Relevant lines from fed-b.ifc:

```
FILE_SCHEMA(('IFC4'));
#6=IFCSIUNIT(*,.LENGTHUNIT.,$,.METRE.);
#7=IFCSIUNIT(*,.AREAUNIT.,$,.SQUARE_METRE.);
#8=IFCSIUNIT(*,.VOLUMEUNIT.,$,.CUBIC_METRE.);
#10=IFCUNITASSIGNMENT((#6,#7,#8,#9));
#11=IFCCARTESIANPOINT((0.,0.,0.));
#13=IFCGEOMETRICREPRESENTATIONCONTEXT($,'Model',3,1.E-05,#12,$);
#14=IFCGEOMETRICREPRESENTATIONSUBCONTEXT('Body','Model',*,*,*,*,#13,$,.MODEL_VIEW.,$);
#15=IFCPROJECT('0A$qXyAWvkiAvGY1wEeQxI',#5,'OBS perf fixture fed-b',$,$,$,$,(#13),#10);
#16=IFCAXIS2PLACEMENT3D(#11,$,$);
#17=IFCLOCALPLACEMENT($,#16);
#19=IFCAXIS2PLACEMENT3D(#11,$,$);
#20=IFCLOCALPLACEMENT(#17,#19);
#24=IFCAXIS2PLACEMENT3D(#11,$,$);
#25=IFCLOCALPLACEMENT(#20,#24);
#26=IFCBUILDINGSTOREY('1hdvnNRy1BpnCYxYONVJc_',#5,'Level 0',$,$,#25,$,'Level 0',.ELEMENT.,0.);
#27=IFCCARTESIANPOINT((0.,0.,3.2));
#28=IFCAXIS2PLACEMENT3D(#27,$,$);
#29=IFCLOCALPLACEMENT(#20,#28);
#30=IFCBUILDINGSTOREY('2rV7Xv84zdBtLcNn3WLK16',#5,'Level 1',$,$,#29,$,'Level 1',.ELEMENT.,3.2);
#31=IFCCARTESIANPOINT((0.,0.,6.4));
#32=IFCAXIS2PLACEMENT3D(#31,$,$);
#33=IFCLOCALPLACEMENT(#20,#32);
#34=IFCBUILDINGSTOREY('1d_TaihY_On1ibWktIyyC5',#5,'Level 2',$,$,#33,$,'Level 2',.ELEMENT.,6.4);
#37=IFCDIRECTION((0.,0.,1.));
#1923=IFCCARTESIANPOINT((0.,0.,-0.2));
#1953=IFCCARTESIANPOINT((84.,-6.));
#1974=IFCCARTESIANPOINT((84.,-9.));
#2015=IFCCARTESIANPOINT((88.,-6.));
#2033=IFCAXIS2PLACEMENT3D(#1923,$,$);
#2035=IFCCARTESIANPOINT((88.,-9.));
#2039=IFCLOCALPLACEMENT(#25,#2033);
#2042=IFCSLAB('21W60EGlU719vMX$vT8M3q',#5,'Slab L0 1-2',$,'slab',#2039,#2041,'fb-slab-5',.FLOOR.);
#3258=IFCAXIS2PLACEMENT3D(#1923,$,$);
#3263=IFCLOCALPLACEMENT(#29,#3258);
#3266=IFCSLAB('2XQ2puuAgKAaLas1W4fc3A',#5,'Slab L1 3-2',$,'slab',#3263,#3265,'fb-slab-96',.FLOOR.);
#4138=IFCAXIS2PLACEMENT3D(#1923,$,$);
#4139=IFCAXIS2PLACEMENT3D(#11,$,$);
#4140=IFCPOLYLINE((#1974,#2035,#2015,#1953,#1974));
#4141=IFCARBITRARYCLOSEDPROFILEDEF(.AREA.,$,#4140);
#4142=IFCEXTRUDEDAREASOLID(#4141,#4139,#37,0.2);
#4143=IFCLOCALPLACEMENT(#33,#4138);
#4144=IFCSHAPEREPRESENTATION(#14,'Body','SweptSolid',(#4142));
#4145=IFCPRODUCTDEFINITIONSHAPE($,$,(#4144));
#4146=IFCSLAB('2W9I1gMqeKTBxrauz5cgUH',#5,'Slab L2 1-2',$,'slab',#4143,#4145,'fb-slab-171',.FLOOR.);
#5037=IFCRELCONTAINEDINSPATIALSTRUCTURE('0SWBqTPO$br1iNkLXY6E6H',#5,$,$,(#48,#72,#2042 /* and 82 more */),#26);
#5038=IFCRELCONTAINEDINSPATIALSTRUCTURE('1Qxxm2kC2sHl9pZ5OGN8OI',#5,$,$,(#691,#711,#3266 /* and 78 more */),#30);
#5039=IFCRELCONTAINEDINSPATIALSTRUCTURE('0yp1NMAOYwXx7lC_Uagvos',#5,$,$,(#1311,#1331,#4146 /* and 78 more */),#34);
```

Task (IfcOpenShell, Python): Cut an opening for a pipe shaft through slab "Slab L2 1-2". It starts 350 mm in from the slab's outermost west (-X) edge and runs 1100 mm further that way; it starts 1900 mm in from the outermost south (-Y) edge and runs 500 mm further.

```python
import numpy as np
import ifcopenshell
import ifcopenshell.api.feature
import ifcopenshell.api.geometry
import ifcopenshell.api.root
import ifcopenshell.geom
import ifcopenshell.util.placement
import ifcopenshell.util.representation
import ifcopenshell.util.shape
import ifcopenshell.util.unit

model = ifcopenshell.open("fed-b.ifc")
unit_scale = ifcopenshell.util.unit.calculate_unit_scale(model)
settings = ifcopenshell.geom.settings()


def volume(element):
    """Net volume in cubic metres, openings subtracted."""
    shape = ifcopenshell.geom.create_shape(settings, element)
    return ifcopenshell.util.shape.get_volume(shape.geometry)


slab = model.by_guid("2W9I1gMqeKTBxrauz5cgUH")
before = volume(slab)

# Extent in the slab's own axes, in metres. The edges named are its -X and -Y sides.
slab_shape = ifcopenshell.geom.create_shape(settings, slab)
vertices = ifcopenshell.util.shape.get_vertices(slab_shape.geometry)
x_min, y_min, bottom = vertices.min(axis=0)
top = vertices[:, 2].max()

opening = ifcopenshell.api.root.create_entity(model, ifc_class="IfcOpeningElement", name="Pipe shaft opening", predefined_type="OPENING")
context = ifcopenshell.util.representation.get_context(model, "Model", "Body", "MODEL_VIEW")
width, depth = 1.1, 0.5
outline = [(0.0, 0.0), (width, 0.0), (width, depth), (0.0, depth), (0.0, 0.0)]
# Overshoot both faces by 50 mm so the cut is clean.
shape = ifcopenshell.api.geometry.add_slab_representation(
    model, context=context, depth=top - bottom + 0.1, polyline=outline
)
ifcopenshell.api.geometry.assign_representation(model, product=opening, representation=shape)

matrix = ifcopenshell.util.placement.get_local_placement(slab.ObjectPlacement)
matrix[:, 3] = matrix @ np.append(np.array([x_min + 0.35, y_min + 1.9, bottom - 0.05]) / unit_scale, 1.0)
ifcopenshell.api.geometry.edit_object_placement(model, product=opening, matrix=matrix, is_si=False)
ifcopenshell.api.feature.add_feature(model, feature=opening, element=slab)

after = volume(slab)

print(f"slab volume {before:.3f} -> {after:.3f} m3")

model.write("fed-b_edited.ifc")
```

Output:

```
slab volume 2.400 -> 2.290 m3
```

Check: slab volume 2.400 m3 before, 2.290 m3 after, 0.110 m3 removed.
